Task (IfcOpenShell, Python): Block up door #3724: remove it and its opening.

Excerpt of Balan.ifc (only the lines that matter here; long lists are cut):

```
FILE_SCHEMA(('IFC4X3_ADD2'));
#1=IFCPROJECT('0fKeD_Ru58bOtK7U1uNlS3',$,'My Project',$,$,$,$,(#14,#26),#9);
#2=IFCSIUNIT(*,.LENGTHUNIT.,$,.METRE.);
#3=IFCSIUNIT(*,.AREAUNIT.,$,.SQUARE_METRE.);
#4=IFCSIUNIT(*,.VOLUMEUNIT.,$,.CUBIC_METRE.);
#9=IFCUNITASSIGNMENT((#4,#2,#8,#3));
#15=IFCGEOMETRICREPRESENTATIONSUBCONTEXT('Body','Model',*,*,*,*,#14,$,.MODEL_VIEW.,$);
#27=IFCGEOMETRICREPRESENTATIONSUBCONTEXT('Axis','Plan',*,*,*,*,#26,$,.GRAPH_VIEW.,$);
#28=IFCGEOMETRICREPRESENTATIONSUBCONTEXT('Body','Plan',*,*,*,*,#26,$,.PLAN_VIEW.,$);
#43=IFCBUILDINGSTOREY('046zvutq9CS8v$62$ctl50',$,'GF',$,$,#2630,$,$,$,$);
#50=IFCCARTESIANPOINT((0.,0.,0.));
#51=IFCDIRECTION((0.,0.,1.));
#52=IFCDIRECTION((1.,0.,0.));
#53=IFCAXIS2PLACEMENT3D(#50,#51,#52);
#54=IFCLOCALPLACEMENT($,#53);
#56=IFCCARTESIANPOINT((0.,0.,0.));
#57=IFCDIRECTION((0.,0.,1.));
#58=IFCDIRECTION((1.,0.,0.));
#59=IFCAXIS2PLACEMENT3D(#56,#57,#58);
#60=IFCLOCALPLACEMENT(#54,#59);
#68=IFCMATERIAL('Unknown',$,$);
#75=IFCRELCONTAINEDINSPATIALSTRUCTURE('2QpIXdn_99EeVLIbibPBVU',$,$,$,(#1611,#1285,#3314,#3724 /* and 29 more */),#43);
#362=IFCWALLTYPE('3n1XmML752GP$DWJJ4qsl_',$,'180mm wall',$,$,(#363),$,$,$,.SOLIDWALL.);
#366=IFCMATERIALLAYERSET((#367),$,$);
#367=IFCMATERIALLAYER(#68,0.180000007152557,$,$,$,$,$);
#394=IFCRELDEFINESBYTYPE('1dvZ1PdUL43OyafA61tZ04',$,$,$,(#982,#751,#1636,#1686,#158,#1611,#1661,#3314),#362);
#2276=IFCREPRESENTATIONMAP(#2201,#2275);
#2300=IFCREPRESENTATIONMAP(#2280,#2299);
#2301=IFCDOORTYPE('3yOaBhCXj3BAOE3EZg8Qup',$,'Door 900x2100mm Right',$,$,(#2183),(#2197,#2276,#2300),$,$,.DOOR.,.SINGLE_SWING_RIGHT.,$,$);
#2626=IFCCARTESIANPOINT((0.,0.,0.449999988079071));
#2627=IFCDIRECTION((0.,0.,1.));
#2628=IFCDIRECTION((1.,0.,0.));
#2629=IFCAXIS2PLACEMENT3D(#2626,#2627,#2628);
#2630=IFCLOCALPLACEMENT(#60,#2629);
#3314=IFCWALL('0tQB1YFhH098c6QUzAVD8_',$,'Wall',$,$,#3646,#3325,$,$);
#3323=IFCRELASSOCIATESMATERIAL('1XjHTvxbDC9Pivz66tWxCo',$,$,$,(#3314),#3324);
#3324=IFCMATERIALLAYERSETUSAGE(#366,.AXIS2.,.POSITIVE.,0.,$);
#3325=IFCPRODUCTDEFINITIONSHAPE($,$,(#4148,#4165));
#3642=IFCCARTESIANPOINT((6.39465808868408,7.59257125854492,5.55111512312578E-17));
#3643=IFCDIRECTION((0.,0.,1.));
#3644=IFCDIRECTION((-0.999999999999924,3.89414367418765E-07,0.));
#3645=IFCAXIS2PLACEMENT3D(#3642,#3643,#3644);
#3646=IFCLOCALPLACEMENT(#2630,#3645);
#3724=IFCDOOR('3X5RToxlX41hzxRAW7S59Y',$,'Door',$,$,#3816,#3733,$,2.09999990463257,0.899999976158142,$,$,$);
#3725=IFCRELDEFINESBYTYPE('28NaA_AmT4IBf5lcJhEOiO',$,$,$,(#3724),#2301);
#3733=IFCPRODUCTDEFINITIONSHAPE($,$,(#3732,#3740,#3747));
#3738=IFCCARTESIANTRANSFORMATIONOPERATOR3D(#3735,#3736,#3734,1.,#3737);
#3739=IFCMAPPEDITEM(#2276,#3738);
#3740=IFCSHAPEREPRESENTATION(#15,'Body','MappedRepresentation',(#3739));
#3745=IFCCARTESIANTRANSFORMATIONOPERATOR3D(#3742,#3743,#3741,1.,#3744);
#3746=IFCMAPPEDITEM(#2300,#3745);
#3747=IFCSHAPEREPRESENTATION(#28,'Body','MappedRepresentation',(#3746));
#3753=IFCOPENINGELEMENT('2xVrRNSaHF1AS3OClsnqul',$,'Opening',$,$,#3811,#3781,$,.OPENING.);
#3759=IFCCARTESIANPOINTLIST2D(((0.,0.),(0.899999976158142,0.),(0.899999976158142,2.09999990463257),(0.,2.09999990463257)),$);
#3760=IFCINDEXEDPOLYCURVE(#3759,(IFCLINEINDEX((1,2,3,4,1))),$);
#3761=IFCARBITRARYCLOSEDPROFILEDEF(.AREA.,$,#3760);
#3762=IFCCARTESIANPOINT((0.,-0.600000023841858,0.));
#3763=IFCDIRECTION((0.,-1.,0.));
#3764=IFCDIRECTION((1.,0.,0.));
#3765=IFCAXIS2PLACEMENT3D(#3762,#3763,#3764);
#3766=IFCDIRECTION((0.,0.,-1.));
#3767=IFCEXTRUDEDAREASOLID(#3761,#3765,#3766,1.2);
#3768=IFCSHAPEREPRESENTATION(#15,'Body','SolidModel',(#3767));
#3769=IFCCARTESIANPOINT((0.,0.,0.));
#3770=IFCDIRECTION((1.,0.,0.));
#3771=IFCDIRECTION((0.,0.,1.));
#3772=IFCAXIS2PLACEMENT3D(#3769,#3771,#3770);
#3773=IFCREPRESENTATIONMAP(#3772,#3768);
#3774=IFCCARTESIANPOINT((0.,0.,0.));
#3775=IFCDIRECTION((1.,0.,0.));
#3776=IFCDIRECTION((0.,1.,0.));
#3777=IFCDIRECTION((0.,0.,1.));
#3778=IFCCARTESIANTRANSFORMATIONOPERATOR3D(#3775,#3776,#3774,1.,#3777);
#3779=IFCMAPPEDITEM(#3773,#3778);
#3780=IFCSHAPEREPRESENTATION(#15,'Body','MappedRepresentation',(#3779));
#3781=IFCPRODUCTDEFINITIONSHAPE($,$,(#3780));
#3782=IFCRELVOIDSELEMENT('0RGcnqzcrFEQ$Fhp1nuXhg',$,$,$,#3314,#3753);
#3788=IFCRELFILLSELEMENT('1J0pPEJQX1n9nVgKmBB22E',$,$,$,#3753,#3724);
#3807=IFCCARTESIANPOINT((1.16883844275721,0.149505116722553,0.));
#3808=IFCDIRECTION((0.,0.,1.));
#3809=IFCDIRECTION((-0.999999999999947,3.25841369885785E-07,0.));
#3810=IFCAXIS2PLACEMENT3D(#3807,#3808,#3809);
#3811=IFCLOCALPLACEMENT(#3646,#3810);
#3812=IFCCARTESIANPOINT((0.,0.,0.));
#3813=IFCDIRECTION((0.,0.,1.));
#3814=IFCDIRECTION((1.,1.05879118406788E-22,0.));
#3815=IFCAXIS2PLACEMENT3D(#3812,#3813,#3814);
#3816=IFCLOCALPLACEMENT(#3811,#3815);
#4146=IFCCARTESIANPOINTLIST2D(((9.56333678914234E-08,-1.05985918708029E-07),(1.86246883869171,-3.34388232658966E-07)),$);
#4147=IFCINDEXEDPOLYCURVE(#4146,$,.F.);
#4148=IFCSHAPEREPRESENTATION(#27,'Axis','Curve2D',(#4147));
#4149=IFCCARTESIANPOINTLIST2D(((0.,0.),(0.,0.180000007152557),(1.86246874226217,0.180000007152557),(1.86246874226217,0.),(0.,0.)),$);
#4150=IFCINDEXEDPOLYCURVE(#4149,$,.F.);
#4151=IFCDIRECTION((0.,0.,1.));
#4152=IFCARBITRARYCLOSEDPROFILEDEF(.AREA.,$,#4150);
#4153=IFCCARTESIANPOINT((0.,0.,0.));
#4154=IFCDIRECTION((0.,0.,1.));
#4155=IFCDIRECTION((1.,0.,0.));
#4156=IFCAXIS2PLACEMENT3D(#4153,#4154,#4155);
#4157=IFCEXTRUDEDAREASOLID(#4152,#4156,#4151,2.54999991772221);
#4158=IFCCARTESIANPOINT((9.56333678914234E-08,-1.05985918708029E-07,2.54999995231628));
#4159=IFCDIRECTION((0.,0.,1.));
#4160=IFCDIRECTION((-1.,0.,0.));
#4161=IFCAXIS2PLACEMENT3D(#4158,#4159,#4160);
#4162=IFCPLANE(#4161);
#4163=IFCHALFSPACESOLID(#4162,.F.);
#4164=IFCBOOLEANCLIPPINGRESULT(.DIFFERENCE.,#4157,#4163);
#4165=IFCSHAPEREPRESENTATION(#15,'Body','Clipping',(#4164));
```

```python
import ifcopenshell
import ifcopenshell.api.feature
import ifcopenshell.api.root
import ifcopenshell.geom
import ifcopenshell.util.shape

model = ifcopenshell.open("Balan.ifc")
settings = ifcopenshell.geom.settings()


def volume(element):
    """Net volume in cubic metres, openings subtracted."""
    shape = ifcopenshell.geom.create_shape(settings, element)
    return ifcopenshell.util.shape.get_volume(shape.geometry)


door = model.by_guid("3X5RToxlX41hzxRAW7S59Y")
opening = door.FillsVoids[0].RelatingOpeningElement
wall = opening.VoidsElements[0].RelatingBuildingElement
before = volume(wall)

ifcopenshell.api.root.remove_product(model, product=door)
ifcopenshell.api.feature.remove_feature(model, feature=opening)

after = volume(wall)

print(f"wall volume {before:.3f} -> {after:.3f} m3")

model.write("Balan_updated.ifc")
```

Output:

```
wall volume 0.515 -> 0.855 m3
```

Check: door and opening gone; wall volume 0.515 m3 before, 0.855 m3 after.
